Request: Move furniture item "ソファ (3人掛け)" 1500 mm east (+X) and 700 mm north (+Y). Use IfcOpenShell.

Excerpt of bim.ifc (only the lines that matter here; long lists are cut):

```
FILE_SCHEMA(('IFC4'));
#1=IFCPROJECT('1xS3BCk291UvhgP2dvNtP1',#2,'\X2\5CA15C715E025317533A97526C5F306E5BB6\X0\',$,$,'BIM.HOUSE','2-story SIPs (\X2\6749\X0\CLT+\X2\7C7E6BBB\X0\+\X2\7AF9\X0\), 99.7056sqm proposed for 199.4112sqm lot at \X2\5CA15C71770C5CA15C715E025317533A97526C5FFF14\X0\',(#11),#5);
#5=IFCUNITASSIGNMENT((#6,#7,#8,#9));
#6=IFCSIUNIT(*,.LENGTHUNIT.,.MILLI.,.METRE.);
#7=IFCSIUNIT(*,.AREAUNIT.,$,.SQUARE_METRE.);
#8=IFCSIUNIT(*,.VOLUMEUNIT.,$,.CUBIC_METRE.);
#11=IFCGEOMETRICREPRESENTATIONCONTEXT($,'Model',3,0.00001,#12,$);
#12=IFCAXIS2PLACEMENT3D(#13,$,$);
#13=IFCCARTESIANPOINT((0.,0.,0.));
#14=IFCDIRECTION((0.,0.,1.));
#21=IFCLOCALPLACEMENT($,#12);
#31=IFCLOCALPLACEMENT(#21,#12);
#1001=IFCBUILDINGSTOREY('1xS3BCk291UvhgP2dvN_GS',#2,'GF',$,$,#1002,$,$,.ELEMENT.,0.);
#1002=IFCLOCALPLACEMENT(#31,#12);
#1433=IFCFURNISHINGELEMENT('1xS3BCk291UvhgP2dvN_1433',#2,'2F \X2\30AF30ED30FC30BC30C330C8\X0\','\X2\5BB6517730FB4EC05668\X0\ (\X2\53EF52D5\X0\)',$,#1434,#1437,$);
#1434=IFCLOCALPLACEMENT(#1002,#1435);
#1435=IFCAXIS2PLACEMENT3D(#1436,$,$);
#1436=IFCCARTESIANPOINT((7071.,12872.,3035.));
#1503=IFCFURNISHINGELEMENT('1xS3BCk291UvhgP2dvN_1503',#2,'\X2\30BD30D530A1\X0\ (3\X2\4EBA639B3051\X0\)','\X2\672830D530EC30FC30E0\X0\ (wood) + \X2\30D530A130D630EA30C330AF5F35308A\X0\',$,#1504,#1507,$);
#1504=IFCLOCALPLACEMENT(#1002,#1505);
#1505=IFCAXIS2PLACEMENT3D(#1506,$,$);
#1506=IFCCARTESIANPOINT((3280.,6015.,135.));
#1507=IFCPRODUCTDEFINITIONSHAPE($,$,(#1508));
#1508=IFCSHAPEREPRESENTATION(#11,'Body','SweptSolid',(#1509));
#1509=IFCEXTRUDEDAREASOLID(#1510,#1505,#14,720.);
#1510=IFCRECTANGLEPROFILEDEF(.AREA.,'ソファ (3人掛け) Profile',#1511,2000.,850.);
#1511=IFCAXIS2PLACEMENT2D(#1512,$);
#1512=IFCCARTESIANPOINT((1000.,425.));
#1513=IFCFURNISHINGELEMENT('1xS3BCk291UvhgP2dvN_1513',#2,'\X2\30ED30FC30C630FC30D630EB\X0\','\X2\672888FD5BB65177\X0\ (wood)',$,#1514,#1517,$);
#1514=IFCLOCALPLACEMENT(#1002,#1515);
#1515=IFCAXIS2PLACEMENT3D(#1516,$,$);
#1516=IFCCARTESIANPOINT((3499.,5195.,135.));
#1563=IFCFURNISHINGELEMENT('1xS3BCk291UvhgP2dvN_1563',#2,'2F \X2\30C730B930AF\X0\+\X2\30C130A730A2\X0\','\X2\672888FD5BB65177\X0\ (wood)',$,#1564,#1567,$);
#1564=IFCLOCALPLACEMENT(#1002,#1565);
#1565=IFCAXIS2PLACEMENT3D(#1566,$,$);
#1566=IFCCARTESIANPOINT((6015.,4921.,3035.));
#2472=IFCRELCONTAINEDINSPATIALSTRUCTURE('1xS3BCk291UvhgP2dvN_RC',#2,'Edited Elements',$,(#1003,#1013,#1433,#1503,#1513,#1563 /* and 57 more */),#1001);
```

```python
import ifcopenshell
import ifcopenshell.api.geometry
import ifcopenshell.util.placement

model = ifcopenshell.open("bim.ifc")

item = model.by_guid("1xS3BCk291UvhgP2dvN_1503")
matrix = ifcopenshell.util.placement.get_local_placement(item.ObjectPlacement)
matrix[0, 3] += 1500.0
matrix[1, 3] += 700.0
ifcopenshell.api.geometry.edit_object_placement(model, product=item, matrix=matrix, is_si=False)

print(ifcopenshell.util.placement.get_local_placement(item.ObjectPlacement).round(3) + 0.0)

model.write("bim_edited.ifc")
```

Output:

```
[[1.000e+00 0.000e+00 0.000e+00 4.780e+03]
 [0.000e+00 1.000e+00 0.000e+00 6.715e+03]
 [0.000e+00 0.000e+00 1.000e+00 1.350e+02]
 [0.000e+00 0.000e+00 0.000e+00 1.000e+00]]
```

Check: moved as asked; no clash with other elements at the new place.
